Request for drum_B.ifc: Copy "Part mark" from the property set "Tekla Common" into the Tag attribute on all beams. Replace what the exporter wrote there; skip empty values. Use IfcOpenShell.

First a look at what the model holds.

```python
import ifcopenshell
import ifcopenshell.util.element

model = ifcopenshell.open("drum_B.ifc")
print(model.schema)
beams = model.by_type("IfcBeam")
print(len(beams), "beams")
for e in beams[:8]:
    source = ifcopenshell.util.element.get_pset(e, "Tekla Common", "Part mark")
    target = e.Tag
    print(e.id(), repr(source), repr(target), sep=" | ")
```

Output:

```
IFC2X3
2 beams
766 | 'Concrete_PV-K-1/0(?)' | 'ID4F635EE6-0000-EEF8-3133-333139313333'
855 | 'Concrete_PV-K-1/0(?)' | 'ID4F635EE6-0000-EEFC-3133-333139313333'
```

```python
import ifcopenshell
import ifcopenshell.util.element

model = ifcopenshell.open("drum_B.ifc")

count = 0
for e in model.by_type("IfcBeam"):
    value = ifcopenshell.util.element.get_pset(e, "Tekla Common", "Part mark")
    current = e.Tag
    if not value or not value.strip() or current == value:
        continue
    e.Tag = value
    count += 1

print(count, "beams updated")

model.write("drum_B-out.ifc")
```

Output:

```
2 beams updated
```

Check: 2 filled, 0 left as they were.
